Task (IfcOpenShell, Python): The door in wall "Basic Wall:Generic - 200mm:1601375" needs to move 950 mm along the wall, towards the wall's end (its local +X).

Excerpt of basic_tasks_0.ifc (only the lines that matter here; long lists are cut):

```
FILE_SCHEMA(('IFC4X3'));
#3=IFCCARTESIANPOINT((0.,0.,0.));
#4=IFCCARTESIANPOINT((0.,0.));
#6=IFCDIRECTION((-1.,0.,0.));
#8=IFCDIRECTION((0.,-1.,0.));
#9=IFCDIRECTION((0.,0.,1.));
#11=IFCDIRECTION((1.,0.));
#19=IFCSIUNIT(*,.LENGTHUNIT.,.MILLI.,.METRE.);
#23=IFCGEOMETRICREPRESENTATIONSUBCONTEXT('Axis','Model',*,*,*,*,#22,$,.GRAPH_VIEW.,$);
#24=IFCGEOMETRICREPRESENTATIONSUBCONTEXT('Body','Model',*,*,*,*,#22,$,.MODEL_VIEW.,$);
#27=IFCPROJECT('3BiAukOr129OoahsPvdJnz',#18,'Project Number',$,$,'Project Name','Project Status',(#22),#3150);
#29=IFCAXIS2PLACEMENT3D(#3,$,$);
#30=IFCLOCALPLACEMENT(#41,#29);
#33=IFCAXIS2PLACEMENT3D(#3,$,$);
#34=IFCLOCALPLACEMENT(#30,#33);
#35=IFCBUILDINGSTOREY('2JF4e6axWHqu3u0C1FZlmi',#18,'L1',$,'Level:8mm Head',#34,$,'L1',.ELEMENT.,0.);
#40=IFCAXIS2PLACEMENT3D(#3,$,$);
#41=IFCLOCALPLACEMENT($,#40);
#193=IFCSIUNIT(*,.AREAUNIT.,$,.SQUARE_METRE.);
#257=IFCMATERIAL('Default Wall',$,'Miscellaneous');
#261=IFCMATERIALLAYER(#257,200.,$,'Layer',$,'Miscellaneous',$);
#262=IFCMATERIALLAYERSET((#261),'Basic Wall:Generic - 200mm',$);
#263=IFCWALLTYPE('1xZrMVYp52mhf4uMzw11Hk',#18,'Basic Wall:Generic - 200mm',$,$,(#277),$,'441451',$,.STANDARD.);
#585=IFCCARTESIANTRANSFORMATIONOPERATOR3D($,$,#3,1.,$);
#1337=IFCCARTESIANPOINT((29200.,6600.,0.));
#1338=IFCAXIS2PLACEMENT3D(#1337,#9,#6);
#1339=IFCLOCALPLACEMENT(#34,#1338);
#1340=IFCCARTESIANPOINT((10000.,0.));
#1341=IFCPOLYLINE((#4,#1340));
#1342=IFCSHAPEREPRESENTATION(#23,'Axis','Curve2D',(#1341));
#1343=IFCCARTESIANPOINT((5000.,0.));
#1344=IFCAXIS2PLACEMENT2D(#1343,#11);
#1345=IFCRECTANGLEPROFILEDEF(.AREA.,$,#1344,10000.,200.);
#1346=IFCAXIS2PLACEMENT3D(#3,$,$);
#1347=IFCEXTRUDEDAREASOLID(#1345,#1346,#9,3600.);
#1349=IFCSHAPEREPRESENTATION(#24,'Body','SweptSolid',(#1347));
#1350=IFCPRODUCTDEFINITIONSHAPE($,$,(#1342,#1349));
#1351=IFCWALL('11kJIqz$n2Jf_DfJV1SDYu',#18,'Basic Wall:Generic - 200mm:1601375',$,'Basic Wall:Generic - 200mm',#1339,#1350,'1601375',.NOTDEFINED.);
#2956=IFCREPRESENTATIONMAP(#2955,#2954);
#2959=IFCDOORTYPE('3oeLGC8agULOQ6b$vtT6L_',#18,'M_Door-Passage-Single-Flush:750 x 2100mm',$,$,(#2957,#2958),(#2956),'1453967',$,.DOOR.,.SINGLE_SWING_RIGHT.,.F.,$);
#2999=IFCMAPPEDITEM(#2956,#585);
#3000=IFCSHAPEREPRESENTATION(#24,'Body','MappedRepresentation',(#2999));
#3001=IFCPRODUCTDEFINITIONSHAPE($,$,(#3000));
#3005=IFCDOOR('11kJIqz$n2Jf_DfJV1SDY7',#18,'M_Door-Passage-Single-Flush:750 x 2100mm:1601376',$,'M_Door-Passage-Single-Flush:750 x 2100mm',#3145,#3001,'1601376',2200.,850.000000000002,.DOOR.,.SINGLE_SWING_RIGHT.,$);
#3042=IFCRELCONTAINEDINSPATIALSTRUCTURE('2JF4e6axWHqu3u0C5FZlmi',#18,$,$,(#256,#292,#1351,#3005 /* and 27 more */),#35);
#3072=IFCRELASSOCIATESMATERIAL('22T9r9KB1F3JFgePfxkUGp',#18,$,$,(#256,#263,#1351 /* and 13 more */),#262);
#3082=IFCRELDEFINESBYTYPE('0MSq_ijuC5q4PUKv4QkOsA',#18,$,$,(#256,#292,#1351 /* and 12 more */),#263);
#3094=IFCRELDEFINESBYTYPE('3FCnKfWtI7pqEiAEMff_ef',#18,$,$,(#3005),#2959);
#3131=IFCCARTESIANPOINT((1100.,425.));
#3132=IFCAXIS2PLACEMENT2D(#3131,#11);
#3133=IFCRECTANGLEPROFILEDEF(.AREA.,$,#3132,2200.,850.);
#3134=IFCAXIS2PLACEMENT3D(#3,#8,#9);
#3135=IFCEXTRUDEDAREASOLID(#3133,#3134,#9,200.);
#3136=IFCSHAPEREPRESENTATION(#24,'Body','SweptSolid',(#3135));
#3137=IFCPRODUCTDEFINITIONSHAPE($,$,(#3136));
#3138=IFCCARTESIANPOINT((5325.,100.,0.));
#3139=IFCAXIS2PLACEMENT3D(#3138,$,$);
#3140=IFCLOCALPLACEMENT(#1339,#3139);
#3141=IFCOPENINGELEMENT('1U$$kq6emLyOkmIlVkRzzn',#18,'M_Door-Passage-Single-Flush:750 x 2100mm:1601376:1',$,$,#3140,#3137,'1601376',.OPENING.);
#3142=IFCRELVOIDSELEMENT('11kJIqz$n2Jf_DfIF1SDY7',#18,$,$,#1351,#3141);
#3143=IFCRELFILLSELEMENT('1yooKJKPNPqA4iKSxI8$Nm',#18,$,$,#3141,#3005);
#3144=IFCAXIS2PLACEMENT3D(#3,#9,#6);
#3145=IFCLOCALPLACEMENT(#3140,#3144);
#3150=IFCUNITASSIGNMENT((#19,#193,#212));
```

```python
import ifcopenshell
import ifcopenshell.api.geometry
import ifcopenshell.util.placement

model = ifcopenshell.open("basic_tasks_0.ifc")

door = model.by_id(3005)
opening = door.FillsVoids[0].RelatingOpeningElement
wall = opening.VoidsElements[0].RelatingBuildingElement

wall_matrix = ifcopenshell.util.placement.get_local_placement(wall.ObjectPlacement)
shift = wall_matrix[:3, 0] * 950.0
before = ifcopenshell.util.placement.get_local_placement(door.ObjectPlacement)[:3, 3].copy()

# The door is placed relative to its opening, so it follows when the opening moves.
matrix = ifcopenshell.util.placement.get_local_placement(opening.ObjectPlacement)
matrix[:3, 3] += shift
ifcopenshell.api.geometry.edit_object_placement(
    model, product=opening, matrix=matrix, is_si=False, should_transform_children=True
)

after = ifcopenshell.util.placement.get_local_placement(door.ObjectPlacement)[:3, 3]
print("door moved by", (after - before).round(3) + 0.0)

model.write("basic_tasks_0_rev.ifc")
```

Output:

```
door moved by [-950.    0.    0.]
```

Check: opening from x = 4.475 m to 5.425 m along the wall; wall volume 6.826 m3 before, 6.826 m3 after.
